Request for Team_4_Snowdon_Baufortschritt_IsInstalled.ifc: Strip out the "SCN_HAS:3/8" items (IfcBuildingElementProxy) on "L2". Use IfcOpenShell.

First a look at what the model holds.

```python
import ifcopenshell
import ifcopenshell.util.element

model = ifcopenshell.open("Team_4_Snowdon_Baufortschritt_IsInstalled.ifc")
print(model.schema)
storey = next(s for s in model.by_type("IfcBuildingStorey") if s.Name == "L2")
proxies = [e for e in ifcopenshell.util.element.get_decomposition(storey) if e.is_a("IfcBuildingElementProxy")]
seen = {}
for e in proxies:
    element_type = ifcopenshell.util.element.get_type(e)
    name = element_type.Name if element_type not in (None, e) else None
    seen[name] = seen.get(name, 0) + 1
for name, count in sorted(seen.items(), key=str):
    print(count, "x", name)
```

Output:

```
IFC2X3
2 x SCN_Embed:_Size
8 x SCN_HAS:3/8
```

```python
import ifcopenshell
import ifcopenshell.api.root
import ifcopenshell.util.element

model = ifcopenshell.open("Team_4_Snowdon_Baufortschritt_IsInstalled.ifc")

storey = next(s for s in model.by_type("IfcBuildingStorey") if s.Name == "L2")
proxies = [e for e in ifcopenshell.util.element.get_decomposition(storey) if e.is_a("IfcBuildingElementProxy")]
targets = [e for e in proxies if (t := ifcopenshell.util.element.get_type(e)) not in (None, e) and t.Name == "SCN_HAS:3/8"]

for e in targets:
    ifcopenshell.api.root.remove_product(model, product=e)
print(len(targets), "removed")

model.write("Team_4_Snowdon_Baufortschritt_IsInstalled_edited.ifc")
```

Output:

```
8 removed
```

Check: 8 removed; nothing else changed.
